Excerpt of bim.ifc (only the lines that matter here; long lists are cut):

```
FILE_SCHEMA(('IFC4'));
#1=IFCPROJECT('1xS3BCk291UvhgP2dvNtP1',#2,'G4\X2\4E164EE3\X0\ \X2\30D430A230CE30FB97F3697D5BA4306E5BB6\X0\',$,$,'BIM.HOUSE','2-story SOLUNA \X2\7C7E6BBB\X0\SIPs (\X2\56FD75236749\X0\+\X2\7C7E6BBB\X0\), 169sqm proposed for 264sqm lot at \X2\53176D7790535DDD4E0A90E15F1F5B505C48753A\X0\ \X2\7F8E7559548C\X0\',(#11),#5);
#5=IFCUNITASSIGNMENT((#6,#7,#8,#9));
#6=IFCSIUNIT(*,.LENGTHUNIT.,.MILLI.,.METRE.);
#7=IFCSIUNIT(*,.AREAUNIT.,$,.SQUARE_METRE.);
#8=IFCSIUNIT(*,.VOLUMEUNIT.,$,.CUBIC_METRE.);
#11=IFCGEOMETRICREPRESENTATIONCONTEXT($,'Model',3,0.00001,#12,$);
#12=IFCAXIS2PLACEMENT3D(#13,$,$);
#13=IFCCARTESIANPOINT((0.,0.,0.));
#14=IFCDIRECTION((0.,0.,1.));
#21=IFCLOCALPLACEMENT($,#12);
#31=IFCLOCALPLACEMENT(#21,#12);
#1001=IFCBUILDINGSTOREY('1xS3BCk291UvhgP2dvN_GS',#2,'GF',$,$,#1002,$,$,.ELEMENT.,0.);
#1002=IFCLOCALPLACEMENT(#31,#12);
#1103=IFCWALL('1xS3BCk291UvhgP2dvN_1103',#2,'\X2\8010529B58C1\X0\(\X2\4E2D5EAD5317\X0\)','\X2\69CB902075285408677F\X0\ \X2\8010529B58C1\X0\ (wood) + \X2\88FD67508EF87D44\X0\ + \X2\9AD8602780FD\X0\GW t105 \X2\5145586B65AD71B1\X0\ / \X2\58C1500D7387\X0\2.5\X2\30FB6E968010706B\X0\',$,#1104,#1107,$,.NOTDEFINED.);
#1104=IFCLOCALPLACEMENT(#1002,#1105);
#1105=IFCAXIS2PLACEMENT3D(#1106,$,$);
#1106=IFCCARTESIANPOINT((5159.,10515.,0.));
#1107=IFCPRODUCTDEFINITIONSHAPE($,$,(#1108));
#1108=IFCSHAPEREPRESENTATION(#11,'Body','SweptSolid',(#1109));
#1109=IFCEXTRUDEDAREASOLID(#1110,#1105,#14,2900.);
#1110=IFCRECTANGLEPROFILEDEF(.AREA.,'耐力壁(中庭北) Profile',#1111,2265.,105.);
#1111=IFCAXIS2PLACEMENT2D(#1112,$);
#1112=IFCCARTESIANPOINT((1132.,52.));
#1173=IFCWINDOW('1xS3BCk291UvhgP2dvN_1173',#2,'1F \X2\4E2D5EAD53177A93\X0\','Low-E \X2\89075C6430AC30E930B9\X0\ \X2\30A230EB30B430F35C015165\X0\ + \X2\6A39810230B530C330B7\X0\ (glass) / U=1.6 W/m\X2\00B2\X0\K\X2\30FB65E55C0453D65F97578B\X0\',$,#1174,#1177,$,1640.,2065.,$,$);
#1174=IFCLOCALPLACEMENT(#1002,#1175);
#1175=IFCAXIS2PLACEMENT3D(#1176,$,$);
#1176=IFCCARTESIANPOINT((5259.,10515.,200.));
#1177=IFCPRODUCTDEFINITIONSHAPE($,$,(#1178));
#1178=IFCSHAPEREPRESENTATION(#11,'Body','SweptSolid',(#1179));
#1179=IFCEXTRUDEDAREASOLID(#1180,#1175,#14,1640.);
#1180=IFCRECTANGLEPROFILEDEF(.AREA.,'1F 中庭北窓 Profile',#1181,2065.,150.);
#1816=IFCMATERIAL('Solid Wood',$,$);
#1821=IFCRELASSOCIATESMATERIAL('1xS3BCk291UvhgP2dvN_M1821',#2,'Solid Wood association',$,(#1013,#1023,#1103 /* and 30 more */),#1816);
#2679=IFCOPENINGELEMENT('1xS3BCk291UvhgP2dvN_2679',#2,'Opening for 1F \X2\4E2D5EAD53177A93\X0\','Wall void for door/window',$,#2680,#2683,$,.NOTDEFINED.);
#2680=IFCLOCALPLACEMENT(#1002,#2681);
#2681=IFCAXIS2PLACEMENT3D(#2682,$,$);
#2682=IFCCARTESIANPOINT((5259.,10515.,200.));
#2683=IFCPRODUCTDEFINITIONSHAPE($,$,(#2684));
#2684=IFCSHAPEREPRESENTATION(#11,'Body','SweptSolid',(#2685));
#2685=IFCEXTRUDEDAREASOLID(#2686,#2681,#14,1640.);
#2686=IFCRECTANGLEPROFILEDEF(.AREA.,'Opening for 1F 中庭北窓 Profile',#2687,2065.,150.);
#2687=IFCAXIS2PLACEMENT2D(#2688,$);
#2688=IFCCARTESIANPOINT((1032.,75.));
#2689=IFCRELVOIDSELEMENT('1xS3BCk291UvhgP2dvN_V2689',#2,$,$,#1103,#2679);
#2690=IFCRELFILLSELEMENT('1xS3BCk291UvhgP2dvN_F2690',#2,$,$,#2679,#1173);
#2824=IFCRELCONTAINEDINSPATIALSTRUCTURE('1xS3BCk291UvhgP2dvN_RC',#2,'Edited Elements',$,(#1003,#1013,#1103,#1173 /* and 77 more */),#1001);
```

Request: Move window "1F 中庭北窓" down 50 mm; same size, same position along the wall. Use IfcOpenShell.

```python
import numpy as np
import ifcopenshell
import ifcopenshell.api.geometry
import ifcopenshell.util.placement
import ifcopenshell.util.unit

model = ifcopenshell.open("bim.ifc")
unit_scale = ifcopenshell.util.unit.calculate_unit_scale(model)

window = model.by_guid("1xS3BCk291UvhgP2dvN_1173")
opening = window.FillsVoids[0].RelatingOpeningElement
dz = -0.05 / unit_scale

shift = np.array([0.0, 0.0, dz])
# The window is not placed relative to its opening, so move both.
for product in (opening, window):
    matrix = ifcopenshell.util.placement.get_local_placement(product.ObjectPlacement)
    matrix[:3, 3] += shift
    ifcopenshell.api.geometry.edit_object_placement(model, product=product, matrix=matrix, is_si=False)

print(f"moved by {dz * unit_scale:+.3f} m")

model.write("bim_updated.ifc")
```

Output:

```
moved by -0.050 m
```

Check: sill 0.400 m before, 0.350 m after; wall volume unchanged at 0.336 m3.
